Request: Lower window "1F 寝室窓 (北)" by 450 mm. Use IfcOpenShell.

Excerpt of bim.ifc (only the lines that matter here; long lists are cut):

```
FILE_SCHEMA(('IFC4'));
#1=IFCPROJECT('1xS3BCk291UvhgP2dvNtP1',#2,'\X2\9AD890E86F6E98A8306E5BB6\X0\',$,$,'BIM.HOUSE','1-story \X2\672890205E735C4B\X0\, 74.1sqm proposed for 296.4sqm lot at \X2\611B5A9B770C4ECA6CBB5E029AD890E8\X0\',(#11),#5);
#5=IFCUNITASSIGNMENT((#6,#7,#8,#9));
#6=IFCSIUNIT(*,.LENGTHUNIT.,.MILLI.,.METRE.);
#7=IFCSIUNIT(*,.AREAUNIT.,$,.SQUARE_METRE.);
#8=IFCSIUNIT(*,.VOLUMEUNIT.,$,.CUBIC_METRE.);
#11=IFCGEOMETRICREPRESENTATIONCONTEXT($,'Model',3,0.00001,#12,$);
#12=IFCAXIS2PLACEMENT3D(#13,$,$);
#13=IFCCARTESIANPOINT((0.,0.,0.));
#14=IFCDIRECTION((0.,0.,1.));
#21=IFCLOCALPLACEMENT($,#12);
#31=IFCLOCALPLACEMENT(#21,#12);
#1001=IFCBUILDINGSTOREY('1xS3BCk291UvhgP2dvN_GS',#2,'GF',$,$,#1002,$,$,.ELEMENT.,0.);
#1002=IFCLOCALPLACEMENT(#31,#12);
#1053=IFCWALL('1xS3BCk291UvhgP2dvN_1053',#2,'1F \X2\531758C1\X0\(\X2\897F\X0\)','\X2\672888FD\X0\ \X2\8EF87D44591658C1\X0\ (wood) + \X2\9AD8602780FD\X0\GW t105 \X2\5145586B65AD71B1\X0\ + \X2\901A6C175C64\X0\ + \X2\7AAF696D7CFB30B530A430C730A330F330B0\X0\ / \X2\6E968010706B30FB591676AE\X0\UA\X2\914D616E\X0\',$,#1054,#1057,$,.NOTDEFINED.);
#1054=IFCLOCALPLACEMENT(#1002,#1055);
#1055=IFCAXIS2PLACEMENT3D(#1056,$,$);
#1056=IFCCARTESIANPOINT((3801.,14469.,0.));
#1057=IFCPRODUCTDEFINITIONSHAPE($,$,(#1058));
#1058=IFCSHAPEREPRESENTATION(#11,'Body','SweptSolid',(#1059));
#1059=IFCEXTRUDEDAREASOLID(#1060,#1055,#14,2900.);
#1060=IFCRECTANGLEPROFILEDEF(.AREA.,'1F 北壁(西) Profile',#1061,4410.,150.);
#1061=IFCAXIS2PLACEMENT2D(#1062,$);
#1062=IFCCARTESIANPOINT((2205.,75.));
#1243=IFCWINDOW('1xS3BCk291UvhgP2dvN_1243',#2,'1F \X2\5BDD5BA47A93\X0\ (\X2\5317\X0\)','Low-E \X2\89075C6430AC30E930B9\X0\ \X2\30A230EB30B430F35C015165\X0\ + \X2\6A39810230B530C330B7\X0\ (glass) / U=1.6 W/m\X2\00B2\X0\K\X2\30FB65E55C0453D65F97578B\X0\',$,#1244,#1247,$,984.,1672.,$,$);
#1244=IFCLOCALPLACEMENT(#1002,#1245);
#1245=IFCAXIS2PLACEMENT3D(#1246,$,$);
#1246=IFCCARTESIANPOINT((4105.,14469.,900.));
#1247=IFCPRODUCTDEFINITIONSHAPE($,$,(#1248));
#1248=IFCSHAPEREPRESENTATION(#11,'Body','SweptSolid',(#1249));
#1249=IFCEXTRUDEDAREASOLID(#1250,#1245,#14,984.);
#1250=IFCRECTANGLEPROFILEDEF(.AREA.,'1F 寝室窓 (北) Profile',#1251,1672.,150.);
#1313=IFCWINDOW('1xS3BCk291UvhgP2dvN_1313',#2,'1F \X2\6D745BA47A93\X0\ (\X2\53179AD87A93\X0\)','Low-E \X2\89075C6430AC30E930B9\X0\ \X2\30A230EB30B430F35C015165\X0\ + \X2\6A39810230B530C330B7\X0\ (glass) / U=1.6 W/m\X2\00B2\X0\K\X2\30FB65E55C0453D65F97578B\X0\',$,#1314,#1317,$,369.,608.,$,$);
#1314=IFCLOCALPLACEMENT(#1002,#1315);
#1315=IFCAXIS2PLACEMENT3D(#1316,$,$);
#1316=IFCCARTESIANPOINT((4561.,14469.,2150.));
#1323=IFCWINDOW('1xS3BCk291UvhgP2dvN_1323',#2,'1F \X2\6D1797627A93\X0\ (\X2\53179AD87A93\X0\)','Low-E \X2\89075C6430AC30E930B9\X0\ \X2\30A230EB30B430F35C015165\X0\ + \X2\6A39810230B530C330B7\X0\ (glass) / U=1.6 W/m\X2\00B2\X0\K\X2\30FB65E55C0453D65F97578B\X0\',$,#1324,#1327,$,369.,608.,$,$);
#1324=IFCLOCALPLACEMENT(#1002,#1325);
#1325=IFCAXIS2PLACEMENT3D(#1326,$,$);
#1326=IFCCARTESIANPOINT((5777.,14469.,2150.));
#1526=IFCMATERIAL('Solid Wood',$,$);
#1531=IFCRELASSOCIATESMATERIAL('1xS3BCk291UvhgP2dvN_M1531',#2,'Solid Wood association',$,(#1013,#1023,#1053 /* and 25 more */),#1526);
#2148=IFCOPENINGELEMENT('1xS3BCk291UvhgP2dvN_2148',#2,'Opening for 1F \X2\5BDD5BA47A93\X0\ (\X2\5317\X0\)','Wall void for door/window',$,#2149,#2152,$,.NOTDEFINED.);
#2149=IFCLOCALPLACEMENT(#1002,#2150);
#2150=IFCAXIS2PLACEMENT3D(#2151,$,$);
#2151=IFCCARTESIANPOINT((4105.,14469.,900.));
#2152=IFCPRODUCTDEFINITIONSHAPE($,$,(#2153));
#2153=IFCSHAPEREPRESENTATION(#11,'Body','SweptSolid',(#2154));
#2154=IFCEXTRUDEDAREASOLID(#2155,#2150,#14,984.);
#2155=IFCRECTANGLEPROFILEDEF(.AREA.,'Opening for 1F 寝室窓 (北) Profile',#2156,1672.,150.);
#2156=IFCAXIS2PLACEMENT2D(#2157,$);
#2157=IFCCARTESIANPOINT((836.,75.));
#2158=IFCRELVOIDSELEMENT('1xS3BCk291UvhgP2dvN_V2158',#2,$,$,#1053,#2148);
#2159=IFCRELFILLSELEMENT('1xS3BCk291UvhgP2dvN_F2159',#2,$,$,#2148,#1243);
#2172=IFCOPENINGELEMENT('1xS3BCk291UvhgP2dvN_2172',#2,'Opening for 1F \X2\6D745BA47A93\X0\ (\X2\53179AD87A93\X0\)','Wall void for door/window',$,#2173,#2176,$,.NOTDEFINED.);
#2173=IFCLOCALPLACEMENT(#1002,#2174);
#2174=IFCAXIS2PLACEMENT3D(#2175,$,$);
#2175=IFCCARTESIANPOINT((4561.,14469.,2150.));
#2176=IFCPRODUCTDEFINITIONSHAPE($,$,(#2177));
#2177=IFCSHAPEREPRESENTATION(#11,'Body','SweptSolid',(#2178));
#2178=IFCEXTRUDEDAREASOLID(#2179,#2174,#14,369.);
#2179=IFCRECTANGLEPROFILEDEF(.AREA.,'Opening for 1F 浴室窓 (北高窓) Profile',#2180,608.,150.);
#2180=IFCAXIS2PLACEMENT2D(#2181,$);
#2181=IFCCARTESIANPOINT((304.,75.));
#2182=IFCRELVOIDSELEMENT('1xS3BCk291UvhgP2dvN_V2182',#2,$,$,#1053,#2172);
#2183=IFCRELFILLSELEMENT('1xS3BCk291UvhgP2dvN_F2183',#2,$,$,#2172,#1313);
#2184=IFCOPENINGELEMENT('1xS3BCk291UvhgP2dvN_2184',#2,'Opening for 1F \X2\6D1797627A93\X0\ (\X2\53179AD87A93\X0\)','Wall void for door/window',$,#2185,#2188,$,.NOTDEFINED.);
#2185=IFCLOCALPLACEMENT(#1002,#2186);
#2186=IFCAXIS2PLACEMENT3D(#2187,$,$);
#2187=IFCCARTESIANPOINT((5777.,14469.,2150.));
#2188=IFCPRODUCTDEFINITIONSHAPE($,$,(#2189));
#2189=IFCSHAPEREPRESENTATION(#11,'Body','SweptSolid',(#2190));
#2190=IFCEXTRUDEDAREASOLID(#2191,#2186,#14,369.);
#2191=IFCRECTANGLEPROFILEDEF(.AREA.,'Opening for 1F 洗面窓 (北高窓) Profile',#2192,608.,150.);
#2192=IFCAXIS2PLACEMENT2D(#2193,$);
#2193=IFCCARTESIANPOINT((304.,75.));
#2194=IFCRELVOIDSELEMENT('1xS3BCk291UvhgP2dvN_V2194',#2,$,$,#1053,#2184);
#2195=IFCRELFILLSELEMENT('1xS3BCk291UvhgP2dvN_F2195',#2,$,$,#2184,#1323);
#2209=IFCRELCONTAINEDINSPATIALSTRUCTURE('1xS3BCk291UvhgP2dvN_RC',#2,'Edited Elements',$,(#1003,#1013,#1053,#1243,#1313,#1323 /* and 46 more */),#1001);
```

```python
import numpy as np
import ifcopenshell
import ifcopenshell.api.geometry
import ifcopenshell.util.placement
import ifcopenshell.util.unit

model = ifcopenshell.open("bim.ifc")
unit_scale = ifcopenshell.util.unit.calculate_unit_scale(model)

window = model.by_guid("1xS3BCk291UvhgP2dvN_1243")
opening = window.FillsVoids[0].RelatingOpeningElement
dz = -0.45 / unit_scale

shift = np.array([0.0, 0.0, dz])
# The window is not placed relative to its opening, so move both.
for product in (opening, window):
    matrix = ifcopenshell.util.placement.get_local_placement(product.ObjectPlacement)
    matrix[:3, 3] += shift
    ifcopenshell.api.geometry.edit_object_placement(model, product=product, matrix=matrix, is_si=False)

print(f"moved by {dz * unit_scale:+.3f} m")

model.write("bim_edited.ifc")
```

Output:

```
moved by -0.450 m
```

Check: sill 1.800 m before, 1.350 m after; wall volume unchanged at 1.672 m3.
